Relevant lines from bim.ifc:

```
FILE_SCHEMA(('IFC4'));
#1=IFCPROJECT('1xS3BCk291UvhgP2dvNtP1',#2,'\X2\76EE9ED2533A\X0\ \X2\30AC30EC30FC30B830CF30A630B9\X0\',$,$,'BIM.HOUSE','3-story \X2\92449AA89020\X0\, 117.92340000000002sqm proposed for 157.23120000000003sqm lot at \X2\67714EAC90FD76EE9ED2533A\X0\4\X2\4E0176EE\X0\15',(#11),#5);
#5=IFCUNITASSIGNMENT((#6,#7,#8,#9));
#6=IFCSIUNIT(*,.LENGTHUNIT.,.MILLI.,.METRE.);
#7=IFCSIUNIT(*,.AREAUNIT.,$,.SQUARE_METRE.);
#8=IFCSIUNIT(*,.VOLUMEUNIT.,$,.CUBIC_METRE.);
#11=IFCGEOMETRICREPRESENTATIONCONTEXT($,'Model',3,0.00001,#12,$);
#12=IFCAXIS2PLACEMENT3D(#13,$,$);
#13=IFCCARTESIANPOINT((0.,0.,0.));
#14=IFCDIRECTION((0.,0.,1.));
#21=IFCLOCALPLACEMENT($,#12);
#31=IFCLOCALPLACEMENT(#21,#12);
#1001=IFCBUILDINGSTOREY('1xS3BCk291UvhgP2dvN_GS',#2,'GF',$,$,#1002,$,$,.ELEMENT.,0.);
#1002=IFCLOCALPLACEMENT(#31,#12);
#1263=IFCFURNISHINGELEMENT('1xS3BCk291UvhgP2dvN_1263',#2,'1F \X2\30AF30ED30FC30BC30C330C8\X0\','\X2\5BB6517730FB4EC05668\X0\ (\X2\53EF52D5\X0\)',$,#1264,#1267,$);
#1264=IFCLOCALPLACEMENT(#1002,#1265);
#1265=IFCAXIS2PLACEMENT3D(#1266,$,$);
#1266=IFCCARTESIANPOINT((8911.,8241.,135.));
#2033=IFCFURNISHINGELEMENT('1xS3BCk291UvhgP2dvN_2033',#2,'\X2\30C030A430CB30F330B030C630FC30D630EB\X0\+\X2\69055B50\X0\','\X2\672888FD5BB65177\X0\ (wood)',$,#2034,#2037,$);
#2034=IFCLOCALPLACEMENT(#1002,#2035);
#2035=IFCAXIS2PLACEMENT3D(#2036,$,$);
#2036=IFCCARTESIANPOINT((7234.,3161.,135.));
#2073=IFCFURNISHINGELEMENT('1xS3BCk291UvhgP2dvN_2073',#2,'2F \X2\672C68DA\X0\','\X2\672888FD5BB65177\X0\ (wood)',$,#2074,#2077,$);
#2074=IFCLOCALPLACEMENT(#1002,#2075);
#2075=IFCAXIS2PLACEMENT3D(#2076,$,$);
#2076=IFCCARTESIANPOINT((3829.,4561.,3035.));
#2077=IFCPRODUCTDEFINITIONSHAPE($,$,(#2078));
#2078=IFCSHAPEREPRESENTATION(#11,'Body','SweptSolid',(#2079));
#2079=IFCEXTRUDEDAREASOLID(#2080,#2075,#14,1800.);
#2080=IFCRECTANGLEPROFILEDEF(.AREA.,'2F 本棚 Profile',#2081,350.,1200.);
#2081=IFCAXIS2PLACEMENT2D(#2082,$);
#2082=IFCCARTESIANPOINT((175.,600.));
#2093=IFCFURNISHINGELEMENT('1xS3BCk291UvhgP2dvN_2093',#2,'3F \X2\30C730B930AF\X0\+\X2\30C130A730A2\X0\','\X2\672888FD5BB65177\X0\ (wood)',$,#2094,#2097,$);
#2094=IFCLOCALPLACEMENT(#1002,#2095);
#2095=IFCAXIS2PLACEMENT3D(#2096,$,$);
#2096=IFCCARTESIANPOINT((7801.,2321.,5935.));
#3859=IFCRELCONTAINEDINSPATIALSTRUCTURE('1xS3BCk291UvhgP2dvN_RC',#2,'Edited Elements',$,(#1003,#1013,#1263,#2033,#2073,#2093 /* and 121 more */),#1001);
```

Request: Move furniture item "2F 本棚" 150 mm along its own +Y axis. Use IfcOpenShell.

```python
import ifcopenshell
import ifcopenshell.api.geometry
import ifcopenshell.util.placement
import ifcopenshell.util.unit

model = ifcopenshell.open("bim.ifc")
unit_scale = ifcopenshell.util.unit.calculate_unit_scale(model)

item = model.by_guid("1xS3BCk291UvhgP2dvN_2073")
matrix = ifcopenshell.util.placement.get_local_placement(item.ObjectPlacement)
matrix[:3, 3] += matrix[:3, 1] * 0.15 / unit_scale
ifcopenshell.api.geometry.edit_object_placement(model, product=item, matrix=matrix, is_si=False)

print(ifcopenshell.util.placement.get_local_placement(item.ObjectPlacement).round(3) + 0.0)

model.write("bim_edited.ifc")
```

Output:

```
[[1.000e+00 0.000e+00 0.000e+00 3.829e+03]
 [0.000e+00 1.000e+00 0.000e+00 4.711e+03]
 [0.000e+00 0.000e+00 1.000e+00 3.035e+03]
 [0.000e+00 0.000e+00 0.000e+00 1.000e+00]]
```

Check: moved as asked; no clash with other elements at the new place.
